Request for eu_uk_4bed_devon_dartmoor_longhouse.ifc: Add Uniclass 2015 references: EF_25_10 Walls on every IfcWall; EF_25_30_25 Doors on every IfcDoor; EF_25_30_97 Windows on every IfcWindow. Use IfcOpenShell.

First a look at what the model holds.

```python
import ifcopenshell

model = ifcopenshell.open("eu_uk_4bed_devon_dartmoor_longhouse.ifc")
print(model.schema)
print("classifications:", [c.Name for c in model.by_type("IfcClassification")])
for ifc_class in ("IfcDoor", "IfcRoof", "IfcStair", "IfcWall", "IfcWindow"):
    print(ifc_class, len(model.by_type(ifc_class)))
```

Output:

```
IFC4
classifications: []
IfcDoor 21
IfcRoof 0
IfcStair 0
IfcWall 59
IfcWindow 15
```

```python
import ifcopenshell
import ifcopenshell.api.classification

model = ifcopenshell.open("eu_uk_4bed_devon_dartmoor_longhouse.ifc")

system = ifcopenshell.api.classification.add_classification(model, classification="Uniclass 2015")

codes = {
    "IfcWall": ("EF_25_10", "Walls"),
    "IfcDoor": ("EF_25_30_25", "Doors"),
    "IfcWindow": ("EF_25_30_97", "Windows"),
}
for ifc_class, (code, name) in codes.items():
    products = model.by_type(ifc_class)
    ifcopenshell.api.classification.add_reference(
        model, products=products, classification=system, identification=code, name=name
    )
    print(code, len(products))

model.write("eu_uk_4bed_devon_dartmoor_longhouse_rev.ifc")
```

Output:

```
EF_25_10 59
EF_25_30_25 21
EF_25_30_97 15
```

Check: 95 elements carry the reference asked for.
